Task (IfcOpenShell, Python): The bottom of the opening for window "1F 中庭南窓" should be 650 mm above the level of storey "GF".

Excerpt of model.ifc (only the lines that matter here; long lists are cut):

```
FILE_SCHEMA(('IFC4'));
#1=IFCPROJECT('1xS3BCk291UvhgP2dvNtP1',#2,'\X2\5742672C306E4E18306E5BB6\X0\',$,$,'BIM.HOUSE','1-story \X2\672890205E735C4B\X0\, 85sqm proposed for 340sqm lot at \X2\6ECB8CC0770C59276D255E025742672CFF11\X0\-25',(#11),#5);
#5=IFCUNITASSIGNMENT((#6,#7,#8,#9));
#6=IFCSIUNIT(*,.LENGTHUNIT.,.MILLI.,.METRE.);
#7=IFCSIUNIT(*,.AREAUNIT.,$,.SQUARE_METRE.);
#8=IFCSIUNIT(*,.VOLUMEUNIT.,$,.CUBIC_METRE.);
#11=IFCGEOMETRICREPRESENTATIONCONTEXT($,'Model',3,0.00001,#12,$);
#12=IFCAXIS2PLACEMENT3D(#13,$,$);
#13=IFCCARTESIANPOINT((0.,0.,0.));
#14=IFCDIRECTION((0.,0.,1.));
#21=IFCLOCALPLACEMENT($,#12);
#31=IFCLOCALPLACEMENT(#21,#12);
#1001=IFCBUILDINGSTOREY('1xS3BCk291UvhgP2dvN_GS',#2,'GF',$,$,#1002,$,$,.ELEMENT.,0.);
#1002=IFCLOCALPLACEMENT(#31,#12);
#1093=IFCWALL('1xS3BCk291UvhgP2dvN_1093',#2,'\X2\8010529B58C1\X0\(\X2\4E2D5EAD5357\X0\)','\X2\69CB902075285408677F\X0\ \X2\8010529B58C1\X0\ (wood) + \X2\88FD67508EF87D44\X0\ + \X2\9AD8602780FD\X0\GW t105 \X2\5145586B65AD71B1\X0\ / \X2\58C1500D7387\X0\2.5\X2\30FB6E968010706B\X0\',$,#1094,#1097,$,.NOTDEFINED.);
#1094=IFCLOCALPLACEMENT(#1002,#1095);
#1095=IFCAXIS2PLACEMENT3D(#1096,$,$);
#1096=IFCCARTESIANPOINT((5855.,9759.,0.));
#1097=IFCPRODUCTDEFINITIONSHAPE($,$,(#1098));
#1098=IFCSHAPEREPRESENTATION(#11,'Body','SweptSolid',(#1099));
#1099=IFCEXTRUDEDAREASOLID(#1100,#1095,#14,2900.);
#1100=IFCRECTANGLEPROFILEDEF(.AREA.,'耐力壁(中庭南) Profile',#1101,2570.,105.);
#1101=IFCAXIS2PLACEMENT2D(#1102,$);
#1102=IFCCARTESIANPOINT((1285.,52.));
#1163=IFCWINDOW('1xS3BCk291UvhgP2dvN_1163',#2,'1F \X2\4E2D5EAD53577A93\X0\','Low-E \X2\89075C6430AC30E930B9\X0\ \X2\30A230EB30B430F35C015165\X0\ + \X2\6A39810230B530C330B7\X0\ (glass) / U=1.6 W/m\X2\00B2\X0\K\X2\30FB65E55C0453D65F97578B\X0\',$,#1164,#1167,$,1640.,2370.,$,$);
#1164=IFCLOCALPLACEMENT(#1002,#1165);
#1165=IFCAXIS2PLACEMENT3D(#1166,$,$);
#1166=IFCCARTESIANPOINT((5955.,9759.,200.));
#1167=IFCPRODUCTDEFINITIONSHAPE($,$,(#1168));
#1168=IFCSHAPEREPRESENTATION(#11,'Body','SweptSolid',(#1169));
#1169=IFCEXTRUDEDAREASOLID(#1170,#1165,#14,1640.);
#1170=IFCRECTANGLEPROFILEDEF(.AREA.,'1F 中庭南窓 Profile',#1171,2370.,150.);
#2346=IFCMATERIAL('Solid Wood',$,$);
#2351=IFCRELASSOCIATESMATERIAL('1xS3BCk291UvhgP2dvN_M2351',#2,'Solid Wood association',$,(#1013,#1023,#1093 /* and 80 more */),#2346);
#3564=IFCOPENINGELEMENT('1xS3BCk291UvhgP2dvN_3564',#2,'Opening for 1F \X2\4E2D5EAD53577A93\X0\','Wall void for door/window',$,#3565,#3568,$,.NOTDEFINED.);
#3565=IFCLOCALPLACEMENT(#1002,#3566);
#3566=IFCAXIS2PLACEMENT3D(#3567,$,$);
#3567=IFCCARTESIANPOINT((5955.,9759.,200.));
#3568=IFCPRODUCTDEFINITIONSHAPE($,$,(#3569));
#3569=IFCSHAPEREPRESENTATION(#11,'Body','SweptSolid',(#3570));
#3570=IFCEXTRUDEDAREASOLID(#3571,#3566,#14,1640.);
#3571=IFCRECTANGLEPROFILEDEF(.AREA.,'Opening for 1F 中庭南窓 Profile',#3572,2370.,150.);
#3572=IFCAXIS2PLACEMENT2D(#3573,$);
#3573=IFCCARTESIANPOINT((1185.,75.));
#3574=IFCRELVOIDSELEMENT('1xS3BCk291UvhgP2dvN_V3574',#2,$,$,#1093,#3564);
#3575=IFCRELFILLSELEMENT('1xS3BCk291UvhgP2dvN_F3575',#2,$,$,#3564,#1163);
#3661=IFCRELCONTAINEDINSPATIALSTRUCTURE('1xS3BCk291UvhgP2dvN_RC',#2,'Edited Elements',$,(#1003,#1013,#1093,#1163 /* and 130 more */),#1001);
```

```python
import numpy as np
import ifcopenshell
import ifcopenshell.api.geometry
import ifcopenshell.geom
import ifcopenshell.util.element
import ifcopenshell.util.placement
import ifcopenshell.util.shape
import ifcopenshell.util.unit

model = ifcopenshell.open("model.ifc")
unit_scale = ifcopenshell.util.unit.calculate_unit_scale(model)

window = model.by_guid("1xS3BCk291UvhgP2dvN_1163")
opening = window.FillsVoids[0].RelatingOpeningElement
storey = ifcopenshell.util.element.get_container(window, ifc_class="IfcBuildingStorey")
level = ifcopenshell.util.placement.get_local_placement(storey.ObjectPlacement)[2, 3]

# The opening's origin need not be at the sill, so measure its lowest point.
shape = ifcopenshell.geom.create_shape(ifcopenshell.geom.settings(), opening)
bottom = ifcopenshell.util.shape.get_shape_bottom_elevation(shape, shape.geometry) / unit_scale
dz = level + 650.0 - bottom

shift = np.array([0.0, 0.0, dz])
# The window is not placed relative to its opening, so move both.
for product in (opening, window):
    matrix = ifcopenshell.util.placement.get_local_placement(product.ObjectPlacement)
    matrix[:3, 3] += shift
    ifcopenshell.api.geometry.edit_object_placement(model, product=product, matrix=matrix, is_si=False)

print(f"moved by {dz * unit_scale:+.3f} m")

model.write("model_v2.ifc")
```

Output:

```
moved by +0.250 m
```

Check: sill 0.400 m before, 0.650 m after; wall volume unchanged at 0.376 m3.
